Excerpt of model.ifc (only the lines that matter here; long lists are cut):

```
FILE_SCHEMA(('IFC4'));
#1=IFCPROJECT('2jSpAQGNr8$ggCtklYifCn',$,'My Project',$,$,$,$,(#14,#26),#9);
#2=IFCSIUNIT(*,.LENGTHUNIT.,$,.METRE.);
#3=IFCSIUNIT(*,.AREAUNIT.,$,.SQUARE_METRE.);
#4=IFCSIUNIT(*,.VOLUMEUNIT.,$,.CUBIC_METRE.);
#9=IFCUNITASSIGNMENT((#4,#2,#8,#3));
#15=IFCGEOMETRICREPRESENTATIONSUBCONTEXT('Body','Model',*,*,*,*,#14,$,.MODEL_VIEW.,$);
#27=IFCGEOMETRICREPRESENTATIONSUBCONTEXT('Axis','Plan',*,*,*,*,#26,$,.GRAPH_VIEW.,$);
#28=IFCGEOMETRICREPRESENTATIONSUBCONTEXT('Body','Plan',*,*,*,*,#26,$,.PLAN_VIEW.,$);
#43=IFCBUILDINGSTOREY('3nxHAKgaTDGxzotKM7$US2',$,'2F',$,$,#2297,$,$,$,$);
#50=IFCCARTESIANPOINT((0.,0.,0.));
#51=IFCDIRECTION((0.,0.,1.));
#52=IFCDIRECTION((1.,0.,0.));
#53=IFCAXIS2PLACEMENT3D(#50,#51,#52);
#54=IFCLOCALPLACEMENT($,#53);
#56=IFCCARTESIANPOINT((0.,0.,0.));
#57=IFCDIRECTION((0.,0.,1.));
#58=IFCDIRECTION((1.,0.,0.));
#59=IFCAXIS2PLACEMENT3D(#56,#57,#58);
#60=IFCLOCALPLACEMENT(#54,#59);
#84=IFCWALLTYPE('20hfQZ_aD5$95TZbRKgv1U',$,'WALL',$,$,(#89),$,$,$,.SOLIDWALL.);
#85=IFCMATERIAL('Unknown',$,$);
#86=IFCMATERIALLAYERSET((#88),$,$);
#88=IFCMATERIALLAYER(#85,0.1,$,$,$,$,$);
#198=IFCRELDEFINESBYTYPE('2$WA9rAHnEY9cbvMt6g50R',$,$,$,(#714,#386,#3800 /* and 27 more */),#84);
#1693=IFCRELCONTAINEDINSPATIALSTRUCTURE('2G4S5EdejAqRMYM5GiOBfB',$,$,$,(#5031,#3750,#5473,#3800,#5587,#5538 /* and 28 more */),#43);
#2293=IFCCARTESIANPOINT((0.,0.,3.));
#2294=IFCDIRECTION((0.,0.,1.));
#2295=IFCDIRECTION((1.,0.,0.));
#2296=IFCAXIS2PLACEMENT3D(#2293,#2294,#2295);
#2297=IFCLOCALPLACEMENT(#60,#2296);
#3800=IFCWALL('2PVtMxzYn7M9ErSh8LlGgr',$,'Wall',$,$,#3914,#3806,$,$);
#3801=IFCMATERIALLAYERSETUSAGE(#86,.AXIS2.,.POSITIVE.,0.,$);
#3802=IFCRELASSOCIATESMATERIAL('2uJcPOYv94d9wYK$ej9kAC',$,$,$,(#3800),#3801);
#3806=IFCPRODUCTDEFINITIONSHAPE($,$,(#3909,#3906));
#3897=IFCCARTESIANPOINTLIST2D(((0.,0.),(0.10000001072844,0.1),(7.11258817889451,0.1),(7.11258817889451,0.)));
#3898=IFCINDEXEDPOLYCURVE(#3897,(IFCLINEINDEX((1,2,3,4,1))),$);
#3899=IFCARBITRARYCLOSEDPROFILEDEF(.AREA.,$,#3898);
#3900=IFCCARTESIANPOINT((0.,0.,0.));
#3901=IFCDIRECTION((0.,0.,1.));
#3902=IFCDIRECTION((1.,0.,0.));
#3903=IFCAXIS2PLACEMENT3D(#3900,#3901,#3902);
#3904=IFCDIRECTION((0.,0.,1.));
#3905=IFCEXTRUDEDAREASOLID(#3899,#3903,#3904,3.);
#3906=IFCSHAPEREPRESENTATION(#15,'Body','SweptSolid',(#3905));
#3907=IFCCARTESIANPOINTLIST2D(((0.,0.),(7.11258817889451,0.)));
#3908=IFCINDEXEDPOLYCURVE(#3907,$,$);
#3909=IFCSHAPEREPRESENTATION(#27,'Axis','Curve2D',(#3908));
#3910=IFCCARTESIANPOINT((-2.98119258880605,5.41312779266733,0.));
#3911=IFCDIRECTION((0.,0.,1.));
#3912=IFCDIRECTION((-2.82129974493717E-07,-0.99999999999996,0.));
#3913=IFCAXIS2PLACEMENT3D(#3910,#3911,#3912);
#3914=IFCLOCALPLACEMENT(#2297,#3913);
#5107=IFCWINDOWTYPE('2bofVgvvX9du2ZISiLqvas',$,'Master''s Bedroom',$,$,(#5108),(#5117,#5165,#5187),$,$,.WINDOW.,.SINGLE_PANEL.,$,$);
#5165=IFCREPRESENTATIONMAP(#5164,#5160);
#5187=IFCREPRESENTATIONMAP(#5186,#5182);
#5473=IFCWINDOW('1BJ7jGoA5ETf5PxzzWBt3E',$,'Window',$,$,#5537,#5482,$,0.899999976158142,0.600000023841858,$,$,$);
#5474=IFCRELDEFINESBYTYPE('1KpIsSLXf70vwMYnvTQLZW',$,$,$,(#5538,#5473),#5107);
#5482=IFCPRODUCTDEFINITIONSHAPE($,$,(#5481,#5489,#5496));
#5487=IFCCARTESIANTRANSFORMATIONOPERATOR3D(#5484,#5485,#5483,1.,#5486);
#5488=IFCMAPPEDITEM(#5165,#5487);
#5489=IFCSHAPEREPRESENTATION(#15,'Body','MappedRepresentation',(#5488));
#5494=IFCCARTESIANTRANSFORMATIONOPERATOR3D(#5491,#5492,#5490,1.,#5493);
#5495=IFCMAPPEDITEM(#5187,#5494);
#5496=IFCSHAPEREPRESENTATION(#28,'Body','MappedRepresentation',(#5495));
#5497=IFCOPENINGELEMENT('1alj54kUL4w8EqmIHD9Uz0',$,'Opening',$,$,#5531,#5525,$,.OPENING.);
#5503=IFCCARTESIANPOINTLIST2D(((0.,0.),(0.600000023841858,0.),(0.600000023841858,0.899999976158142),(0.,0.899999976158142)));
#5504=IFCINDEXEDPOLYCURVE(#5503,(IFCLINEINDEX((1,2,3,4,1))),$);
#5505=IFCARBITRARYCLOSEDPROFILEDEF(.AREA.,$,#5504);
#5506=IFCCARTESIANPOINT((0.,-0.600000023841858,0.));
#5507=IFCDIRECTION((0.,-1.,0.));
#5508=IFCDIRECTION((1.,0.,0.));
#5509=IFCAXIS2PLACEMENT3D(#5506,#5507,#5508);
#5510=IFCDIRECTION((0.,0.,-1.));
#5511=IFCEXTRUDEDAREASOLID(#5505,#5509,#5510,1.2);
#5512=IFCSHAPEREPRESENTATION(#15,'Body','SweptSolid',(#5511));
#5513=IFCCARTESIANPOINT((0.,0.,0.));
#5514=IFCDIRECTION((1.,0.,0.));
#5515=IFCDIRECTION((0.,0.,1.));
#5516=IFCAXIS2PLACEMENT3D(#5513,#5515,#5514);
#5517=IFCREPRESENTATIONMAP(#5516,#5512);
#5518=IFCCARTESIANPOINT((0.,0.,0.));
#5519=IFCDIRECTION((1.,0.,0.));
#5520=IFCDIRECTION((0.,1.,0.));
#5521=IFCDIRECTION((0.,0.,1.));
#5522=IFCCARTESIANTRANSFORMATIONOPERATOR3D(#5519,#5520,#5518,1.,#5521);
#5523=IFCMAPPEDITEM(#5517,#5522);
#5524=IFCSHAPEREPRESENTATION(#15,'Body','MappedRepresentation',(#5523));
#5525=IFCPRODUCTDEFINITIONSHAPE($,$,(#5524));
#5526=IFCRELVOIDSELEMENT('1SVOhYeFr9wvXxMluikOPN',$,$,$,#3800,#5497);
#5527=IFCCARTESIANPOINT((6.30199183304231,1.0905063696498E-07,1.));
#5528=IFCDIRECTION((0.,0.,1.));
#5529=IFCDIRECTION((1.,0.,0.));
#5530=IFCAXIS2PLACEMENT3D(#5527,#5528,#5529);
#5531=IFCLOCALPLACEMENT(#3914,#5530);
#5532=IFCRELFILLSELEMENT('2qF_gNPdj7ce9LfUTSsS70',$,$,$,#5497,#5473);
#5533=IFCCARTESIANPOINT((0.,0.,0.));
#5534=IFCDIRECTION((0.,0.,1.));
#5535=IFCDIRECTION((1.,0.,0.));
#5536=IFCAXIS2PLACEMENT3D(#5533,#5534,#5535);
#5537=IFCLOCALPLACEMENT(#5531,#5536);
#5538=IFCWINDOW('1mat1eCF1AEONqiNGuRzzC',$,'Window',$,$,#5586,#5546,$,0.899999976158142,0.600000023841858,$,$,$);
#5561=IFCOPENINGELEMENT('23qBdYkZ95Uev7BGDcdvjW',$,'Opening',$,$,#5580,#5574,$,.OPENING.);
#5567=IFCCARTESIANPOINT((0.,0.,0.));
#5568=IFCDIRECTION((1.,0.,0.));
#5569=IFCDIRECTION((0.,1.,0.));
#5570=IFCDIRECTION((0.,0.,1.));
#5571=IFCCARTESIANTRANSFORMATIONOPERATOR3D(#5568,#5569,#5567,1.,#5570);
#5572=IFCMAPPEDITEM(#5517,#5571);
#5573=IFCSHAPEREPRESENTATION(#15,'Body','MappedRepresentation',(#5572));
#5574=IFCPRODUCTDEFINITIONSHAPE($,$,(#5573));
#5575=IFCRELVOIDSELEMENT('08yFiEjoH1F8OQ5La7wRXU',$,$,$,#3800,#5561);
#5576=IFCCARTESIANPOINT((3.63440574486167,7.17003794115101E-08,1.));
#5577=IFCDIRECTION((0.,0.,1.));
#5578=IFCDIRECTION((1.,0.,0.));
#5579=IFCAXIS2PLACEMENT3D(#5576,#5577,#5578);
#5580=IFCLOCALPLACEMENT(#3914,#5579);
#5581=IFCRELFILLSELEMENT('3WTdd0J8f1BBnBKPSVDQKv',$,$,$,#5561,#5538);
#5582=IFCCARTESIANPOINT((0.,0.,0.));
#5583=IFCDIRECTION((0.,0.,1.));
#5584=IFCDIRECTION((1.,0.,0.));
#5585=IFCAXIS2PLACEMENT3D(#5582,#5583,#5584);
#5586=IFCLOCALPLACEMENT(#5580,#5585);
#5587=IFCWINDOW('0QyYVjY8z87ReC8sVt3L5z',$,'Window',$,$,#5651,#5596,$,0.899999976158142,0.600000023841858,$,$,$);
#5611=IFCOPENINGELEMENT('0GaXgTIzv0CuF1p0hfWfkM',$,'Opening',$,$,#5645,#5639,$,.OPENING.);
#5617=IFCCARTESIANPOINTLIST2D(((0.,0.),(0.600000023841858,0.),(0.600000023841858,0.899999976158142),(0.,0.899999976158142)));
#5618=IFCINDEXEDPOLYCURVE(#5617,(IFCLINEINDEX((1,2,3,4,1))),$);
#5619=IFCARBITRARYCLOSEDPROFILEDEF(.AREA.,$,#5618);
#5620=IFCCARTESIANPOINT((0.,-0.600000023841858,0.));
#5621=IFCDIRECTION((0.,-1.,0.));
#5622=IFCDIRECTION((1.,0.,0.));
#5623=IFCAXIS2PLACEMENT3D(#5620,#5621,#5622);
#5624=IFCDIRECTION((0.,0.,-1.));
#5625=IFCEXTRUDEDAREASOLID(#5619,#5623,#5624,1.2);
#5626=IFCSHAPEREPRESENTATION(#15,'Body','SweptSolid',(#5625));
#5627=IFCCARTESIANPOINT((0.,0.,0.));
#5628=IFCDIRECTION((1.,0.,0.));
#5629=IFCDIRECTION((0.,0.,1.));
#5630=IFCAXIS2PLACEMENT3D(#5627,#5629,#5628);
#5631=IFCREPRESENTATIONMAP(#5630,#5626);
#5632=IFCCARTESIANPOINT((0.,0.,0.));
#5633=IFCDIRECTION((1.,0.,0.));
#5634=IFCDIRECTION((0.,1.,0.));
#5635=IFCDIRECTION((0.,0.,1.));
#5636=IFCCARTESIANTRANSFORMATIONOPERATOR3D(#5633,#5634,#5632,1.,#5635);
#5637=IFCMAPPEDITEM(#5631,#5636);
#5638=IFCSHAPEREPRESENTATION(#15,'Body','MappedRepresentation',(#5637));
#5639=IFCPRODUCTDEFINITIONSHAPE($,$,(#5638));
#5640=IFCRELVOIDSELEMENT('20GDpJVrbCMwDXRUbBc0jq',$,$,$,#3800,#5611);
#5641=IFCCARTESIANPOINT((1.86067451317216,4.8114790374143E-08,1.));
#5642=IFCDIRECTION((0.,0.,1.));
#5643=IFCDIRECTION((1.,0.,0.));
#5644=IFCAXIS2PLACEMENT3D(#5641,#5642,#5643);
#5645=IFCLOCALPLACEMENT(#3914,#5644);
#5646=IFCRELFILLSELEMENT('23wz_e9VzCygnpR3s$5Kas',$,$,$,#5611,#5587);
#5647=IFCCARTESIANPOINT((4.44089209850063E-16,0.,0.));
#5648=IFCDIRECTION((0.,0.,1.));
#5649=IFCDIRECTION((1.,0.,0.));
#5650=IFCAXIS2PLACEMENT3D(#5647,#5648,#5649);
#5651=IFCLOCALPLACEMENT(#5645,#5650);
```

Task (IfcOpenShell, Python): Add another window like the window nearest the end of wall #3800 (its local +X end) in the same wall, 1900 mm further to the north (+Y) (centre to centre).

```python
import ifcopenshell
import ifcopenshell.api.feature
import ifcopenshell.api.geometry
import ifcopenshell.api.root
import ifcopenshell.geom
import ifcopenshell.util.element
import ifcopenshell.util.placement
import ifcopenshell.util.shape
import ifcopenshell.util.unit

model = ifcopenshell.open("model.ifc")
unit_scale = ifcopenshell.util.unit.calculate_unit_scale(model)
settings = ifcopenshell.geom.settings()


def volume(element):
    """Net volume in cubic metres, openings subtracted."""
    shape = ifcopenshell.geom.create_shape(settings, element)
    return ifcopenshell.util.shape.get_volume(shape.geometry)


window = model.by_guid("1BJ7jGoA5ETf5PxzzWBt3E")
opening = window.FillsVoids[0].RelatingOpeningElement
wall = opening.VoidsElements[0].RelatingBuildingElement
before = volume(wall)
shift = ifcopenshell.util.placement.get_local_placement(wall.ObjectPlacement)[:3, 0] * -1.9 / unit_scale

# copy_class copies the void relationship, type, container and properties, but no geometry.
new_opening = ifcopenshell.api.root.copy_class(model, product=opening)
new_opening.Representation = ifcopenshell.util.element.copy_deep(
    model, opening.Representation, exclude=["IfcGeometricRepresentationContext", "IfcRepresentationMap"]
)
new_window = ifcopenshell.api.root.copy_class(model, product=window)
new_window.Representation = ifcopenshell.util.element.copy_deep(
    model, window.Representation, exclude=["IfcGeometricRepresentationContext", "IfcRepresentationMap"]
)
ifcopenshell.api.feature.add_filling(model, opening=new_opening, element=new_window)

for old, new in ((opening, new_opening), (window, new_window)):
    matrix = ifcopenshell.util.placement.get_local_placement(old.ObjectPlacement)
    matrix[:3, 3] += shift
    ifcopenshell.api.geometry.edit_object_placement(model, product=new, matrix=matrix, is_si=False)

after = volume(wall)

print(f"wall volume {before:.3f} -> {after:.3f} m3")

model.write("model_edited.ifc")
```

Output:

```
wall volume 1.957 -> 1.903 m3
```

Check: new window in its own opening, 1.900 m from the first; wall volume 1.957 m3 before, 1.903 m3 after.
